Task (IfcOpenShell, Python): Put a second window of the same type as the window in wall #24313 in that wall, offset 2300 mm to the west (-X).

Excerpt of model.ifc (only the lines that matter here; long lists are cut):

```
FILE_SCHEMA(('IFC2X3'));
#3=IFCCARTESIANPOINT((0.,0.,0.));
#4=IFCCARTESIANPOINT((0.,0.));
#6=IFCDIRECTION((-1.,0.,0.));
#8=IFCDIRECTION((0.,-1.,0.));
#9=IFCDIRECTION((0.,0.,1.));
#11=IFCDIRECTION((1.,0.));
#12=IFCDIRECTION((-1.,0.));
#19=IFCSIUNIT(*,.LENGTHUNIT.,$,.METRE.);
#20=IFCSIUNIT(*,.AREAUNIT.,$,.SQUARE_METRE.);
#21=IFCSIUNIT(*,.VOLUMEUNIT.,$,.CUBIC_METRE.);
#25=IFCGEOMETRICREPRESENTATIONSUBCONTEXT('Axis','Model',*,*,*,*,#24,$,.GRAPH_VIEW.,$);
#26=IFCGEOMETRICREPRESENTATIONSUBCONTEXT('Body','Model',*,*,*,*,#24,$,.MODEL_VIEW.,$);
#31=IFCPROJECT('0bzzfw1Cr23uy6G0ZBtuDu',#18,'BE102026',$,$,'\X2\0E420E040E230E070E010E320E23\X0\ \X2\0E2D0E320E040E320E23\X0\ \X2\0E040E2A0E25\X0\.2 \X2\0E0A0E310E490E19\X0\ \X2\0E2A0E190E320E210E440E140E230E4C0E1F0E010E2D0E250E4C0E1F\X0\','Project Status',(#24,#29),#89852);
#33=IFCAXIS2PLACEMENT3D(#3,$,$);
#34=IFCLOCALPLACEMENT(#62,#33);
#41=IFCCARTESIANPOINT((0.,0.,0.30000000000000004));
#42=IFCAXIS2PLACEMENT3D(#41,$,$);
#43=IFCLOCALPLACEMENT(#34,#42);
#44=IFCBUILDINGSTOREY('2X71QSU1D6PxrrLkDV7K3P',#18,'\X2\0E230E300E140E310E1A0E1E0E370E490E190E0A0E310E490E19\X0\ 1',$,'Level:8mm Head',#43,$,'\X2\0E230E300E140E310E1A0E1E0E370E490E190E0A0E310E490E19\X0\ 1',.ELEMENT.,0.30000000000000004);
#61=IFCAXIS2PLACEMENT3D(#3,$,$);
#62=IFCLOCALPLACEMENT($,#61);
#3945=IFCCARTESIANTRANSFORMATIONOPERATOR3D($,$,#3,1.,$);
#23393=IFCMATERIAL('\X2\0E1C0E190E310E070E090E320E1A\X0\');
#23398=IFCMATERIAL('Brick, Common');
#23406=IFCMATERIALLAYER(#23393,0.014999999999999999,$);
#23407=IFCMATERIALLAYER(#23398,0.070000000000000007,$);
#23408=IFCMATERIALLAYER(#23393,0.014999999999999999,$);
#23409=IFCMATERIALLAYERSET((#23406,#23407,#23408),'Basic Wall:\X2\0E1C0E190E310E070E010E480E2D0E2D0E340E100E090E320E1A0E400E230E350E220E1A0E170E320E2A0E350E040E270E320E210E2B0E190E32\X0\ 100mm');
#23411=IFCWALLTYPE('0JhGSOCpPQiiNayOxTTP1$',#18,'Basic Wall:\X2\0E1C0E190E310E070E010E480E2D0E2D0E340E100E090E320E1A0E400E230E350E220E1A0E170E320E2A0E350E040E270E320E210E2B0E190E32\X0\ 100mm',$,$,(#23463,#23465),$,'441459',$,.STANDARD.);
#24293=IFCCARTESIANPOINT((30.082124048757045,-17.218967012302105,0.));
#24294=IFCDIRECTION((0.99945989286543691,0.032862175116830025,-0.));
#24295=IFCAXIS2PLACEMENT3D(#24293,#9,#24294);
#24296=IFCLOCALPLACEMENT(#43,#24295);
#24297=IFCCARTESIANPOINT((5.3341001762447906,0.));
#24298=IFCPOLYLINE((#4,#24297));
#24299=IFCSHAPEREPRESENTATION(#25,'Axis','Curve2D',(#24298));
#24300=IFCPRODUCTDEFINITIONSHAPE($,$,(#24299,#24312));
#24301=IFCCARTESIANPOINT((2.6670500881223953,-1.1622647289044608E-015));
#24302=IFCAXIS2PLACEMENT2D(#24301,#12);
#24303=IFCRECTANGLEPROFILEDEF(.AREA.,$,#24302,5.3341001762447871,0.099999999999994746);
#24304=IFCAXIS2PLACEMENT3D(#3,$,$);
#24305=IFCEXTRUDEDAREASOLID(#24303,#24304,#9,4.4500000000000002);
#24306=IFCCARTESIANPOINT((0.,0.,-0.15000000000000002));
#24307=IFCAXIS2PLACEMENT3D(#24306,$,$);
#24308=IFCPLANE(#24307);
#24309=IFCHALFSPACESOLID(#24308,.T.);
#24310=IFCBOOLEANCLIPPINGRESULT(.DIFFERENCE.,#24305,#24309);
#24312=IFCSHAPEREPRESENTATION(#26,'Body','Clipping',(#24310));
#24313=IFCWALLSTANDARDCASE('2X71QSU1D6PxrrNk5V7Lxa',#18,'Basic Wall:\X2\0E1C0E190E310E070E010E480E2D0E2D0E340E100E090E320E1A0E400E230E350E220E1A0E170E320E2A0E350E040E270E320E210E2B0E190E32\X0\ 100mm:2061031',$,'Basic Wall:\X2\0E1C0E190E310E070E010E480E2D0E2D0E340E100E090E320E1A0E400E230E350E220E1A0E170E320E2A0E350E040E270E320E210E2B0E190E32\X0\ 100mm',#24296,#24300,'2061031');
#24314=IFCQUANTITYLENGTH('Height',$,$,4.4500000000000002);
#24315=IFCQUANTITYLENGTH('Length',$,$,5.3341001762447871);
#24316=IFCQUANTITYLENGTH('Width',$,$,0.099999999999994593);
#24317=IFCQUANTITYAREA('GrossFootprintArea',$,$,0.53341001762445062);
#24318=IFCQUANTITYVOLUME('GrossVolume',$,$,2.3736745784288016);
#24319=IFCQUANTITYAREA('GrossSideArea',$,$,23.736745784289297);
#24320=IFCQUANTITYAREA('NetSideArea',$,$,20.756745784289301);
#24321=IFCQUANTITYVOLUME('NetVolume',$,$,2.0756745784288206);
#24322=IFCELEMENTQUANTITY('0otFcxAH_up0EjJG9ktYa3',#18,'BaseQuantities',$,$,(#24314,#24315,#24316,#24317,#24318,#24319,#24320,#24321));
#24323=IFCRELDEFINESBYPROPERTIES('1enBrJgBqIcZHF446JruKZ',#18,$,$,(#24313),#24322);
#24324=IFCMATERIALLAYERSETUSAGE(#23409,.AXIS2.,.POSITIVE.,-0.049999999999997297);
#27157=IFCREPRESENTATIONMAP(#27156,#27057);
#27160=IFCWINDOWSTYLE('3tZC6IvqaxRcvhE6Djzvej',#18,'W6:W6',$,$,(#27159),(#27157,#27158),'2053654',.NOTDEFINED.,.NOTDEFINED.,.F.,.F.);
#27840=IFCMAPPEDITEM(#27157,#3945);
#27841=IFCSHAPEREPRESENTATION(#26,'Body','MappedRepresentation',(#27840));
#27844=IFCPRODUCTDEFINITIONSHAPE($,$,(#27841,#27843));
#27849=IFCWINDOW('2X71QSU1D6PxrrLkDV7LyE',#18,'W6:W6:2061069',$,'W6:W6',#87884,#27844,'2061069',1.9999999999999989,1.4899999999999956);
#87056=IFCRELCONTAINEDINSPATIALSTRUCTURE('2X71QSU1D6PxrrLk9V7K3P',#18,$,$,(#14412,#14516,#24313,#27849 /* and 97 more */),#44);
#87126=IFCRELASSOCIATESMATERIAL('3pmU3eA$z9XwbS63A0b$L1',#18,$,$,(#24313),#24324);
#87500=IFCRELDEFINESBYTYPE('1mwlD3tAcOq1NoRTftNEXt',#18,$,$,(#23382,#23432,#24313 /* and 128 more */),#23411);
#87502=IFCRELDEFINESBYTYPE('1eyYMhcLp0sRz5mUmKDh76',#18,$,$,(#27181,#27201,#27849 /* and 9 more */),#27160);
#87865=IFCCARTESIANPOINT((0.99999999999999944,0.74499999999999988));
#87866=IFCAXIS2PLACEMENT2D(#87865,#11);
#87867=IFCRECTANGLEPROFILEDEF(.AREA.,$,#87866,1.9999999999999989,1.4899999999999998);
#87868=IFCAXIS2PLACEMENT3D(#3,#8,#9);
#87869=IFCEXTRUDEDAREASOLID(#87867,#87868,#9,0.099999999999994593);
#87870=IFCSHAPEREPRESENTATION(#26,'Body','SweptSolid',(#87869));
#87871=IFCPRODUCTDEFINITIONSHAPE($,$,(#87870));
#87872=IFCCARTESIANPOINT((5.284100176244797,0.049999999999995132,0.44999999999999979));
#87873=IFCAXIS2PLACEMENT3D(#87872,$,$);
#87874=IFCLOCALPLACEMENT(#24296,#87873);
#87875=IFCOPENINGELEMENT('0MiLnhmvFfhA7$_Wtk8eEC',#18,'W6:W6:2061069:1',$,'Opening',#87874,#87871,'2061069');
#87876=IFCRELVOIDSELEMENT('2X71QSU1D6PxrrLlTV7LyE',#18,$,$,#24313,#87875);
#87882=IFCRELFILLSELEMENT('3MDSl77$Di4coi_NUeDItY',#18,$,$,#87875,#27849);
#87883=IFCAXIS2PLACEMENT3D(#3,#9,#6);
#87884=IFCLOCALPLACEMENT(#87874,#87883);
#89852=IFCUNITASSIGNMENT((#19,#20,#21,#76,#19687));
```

```python
import ifcopenshell
import ifcopenshell.api.feature
import ifcopenshell.api.geometry
import ifcopenshell.api.pset
import ifcopenshell.api.root
import ifcopenshell.geom
import ifcopenshell.util.element
import ifcopenshell.util.placement
import ifcopenshell.util.shape
import ifcopenshell.util.unit

model = ifcopenshell.open("model.ifc")
unit_scale = ifcopenshell.util.unit.calculate_unit_scale(model)
area_scale = ifcopenshell.util.unit.calculate_unit_scale(model, "AREAUNIT")
volume_scale = ifcopenshell.util.unit.calculate_unit_scale(model, "VOLUMEUNIT")
settings = ifcopenshell.geom.settings()


def volume(element):
    """Net volume in cubic metres, openings subtracted."""
    shape = ifcopenshell.geom.create_shape(settings, element)
    return ifcopenshell.util.shape.get_volume(shape.geometry)


def reuse_history(source, copy):
    """copy_class also copies each property set's owner history, people and application; keep the originals."""
    for rel in copy.IsDefinedBy:
        if rel.is_a("IfcRelDefinesByProperties") and (history := rel.RelatingPropertyDefinition.OwnerHistory):
            rel.RelatingPropertyDefinition.OwnerHistory = source.OwnerHistory
            ifcopenshell.util.element.remove_deep2(model, history)


window = model.by_guid("2X71QSU1D6PxrrLkDV7LyE")
opening = window.FillsVoids[0].RelatingOpeningElement
wall = opening.VoidsElements[0].RelatingBuildingElement
before = volume(wall)
shift = ifcopenshell.util.placement.get_local_placement(wall.ObjectPlacement)[:3, 0] * -2.3 / unit_scale

# copy_class copies the void relationship, type, container and properties, but no geometry.
new_opening = ifcopenshell.api.root.copy_class(model, product=opening)
new_opening.Representation = ifcopenshell.util.element.copy_deep(
    model, opening.Representation, exclude=["IfcGeometricRepresentationContext", "IfcRepresentationMap"]
)
new_opening.Name = "W6:W6"
new_opening.Tag = None
reuse_history(opening, new_opening)
new_window = ifcopenshell.api.root.copy_class(model, product=window)
new_window.Representation = ifcopenshell.util.element.copy_deep(
    model, window.Representation, exclude=["IfcGeometricRepresentationContext", "IfcRepresentationMap"]
)
new_window.Name = "W6:W6"
new_window.Tag = None
reuse_history(window, new_window)
fills = ifcopenshell.api.feature.add_filling(model, opening=new_opening, element=new_window)
fills.OwnerHistory = new_window.OwnerHistory  # required in IFC2X3

for old, new in ((opening, new_opening), (window, new_window)):
    matrix = ifcopenshell.util.placement.get_local_placement(old.ObjectPlacement)
    matrix[:3, 3] += shift
    ifcopenshell.api.geometry.edit_object_placement(model, product=new, matrix=matrix, is_si=False)

after = volume(wall)
thickness = 0.1  # wall thickness in metres

# Update the wall's stored quantities.
qto = model.by_id(ifcopenshell.util.element.get_pset(wall, "BaseQuantities", should_inherit=False)["id"])
ifcopenshell.api.pset.edit_qto(model, qto=qto, properties={
    "NetSideArea": after / thickness / area_scale,
    "NetVolume": after / volume_scale,
})

print(f"wall volume {before:.3f} -> {after:.3f} m3")

model.write("model_rev.ifc")
```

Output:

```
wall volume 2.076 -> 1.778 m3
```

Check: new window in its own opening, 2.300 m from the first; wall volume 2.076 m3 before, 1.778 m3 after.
